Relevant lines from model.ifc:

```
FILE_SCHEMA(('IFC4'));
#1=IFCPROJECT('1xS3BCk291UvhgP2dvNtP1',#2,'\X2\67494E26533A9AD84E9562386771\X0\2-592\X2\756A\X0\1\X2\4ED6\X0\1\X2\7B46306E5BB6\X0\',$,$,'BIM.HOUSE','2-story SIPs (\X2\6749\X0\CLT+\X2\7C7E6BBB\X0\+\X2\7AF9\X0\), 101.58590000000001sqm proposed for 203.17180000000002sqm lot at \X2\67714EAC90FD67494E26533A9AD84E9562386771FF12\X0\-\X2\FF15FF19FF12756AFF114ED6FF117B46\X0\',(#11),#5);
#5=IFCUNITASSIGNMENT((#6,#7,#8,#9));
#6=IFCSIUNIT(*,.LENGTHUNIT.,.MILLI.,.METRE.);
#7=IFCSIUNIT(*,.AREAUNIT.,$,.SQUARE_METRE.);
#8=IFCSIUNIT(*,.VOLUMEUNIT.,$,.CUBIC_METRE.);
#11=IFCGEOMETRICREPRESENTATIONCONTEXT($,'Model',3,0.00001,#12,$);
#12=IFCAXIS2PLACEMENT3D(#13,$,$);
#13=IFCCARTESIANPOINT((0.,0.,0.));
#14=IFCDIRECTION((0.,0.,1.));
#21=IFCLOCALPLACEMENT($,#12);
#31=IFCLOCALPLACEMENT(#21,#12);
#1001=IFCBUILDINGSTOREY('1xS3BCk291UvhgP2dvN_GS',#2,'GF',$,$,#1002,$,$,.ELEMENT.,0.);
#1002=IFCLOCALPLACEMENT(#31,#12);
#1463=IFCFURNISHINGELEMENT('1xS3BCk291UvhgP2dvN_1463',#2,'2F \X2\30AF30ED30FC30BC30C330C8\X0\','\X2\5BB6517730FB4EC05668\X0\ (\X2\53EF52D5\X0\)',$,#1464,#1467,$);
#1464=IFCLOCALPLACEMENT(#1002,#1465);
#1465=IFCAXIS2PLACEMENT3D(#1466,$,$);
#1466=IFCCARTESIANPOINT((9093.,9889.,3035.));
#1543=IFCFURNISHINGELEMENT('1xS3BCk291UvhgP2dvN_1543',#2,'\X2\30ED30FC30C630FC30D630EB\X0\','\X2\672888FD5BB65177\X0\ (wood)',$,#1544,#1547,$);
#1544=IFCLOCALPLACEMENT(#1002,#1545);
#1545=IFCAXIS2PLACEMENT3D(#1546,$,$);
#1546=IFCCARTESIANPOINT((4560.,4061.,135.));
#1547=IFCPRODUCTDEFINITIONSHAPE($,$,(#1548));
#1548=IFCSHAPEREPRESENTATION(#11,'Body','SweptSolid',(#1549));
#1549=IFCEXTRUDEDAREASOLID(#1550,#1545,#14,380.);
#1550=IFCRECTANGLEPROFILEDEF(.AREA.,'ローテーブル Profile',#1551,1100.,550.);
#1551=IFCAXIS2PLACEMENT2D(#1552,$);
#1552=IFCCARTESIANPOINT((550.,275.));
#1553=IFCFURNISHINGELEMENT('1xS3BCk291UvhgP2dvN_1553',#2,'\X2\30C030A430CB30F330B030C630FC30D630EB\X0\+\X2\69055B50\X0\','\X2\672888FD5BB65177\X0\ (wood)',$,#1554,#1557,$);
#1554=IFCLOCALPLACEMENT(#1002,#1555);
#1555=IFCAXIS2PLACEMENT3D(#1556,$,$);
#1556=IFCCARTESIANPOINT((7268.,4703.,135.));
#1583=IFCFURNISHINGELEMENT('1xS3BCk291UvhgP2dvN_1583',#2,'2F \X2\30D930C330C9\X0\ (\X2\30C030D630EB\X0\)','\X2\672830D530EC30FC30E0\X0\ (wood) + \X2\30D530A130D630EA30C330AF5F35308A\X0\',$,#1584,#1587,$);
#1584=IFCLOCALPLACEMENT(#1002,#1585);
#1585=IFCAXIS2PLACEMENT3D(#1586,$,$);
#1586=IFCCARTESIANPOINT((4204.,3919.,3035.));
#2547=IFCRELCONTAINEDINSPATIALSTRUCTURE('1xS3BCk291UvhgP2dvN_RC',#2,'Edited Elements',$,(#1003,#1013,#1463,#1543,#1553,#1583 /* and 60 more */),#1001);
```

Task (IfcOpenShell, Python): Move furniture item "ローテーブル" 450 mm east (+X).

```python
import ifcopenshell
import ifcopenshell.api.geometry
import ifcopenshell.util.placement

model = ifcopenshell.open("model.ifc")

item = model.by_id(1543)
matrix = ifcopenshell.util.placement.get_local_placement(item.ObjectPlacement)
matrix[0, 3] += 450.0
ifcopenshell.api.geometry.edit_object_placement(model, product=item, matrix=matrix, is_si=False)

print(ifcopenshell.util.placement.get_local_placement(item.ObjectPlacement).round(3) + 0.0)

model.write("model_v2.ifc")
```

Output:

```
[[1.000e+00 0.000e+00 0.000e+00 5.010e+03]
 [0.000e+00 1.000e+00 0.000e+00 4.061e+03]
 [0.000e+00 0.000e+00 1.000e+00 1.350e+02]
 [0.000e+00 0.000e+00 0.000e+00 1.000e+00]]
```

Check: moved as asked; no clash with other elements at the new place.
